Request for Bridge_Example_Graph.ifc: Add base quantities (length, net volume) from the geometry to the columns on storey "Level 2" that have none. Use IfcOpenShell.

First a look at what the model holds.

```python
import ifcopenshell
import ifcopenshell.util.element
import ifcopenshell.util.unit

model = ifcopenshell.open("Bridge_Example_Graph.ifc")
print(model.schema)
for unit_type in ("LENGTHUNIT", "AREAUNIT", "VOLUMEUNIT"):
    print(unit_type, ifcopenshell.util.unit.calculate_unit_scale(model, unit_type))
storey = next(s for s in model.by_type("IfcBuildingStorey") if s.Name == "Level 2")
columns = [e for e in ifcopenshell.util.element.get_decomposition(storey) if e.is_a("IfcColumn")]
for e in sorted(columns, key=lambda e: e.id()):
    print(e.id(), e.is_a(), e.Name, list(ifcopenshell.util.element.get_psets(e, qtos_only=True)), sep=" | ")
```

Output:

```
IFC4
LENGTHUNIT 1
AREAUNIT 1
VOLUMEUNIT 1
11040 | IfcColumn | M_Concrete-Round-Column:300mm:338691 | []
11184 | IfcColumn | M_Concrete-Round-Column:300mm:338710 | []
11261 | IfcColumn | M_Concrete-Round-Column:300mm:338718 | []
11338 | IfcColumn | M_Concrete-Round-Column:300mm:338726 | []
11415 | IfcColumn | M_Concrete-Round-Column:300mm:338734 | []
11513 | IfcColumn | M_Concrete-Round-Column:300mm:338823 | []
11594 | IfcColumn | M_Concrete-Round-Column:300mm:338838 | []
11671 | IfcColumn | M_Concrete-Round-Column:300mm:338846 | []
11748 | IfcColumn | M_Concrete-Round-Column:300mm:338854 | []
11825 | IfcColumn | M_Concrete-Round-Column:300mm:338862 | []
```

```python
import ifcopenshell
import ifcopenshell.api.pset
import ifcopenshell.geom
import ifcopenshell.util.element
import ifcopenshell.util.shape
import ifcopenshell.util.unit

model = ifcopenshell.open("Bridge_Example_Graph.ifc")
unit_scale = ifcopenshell.util.unit.calculate_unit_scale(model)
volume_scale = ifcopenshell.util.unit.calculate_unit_scale(model, "VOLUMEUNIT")
settings = ifcopenshell.geom.settings()

storey = next(s for s in model.by_type("IfcBuildingStorey") if s.Name == "Level 2")
columns = [e for e in ifcopenshell.util.element.get_decomposition(storey) if e.is_a("IfcColumn")]

for e in sorted(columns, key=lambda e: e.id()):
    if ifcopenshell.util.element.get_psets(e, qtos_only=True, should_inherit=False):
        continue
    # Geometry comes back in metres, in the element's own axes.
    shape = ifcopenshell.geom.create_shape(settings, e)
    values = {
        "Length": ifcopenshell.util.shape.get_z(shape.geometry) / unit_scale,
        "NetVolume": ifcopenshell.util.shape.get_volume(shape.geometry) / volume_scale,
    }
    qto = ifcopenshell.api.pset.add_qto(model, product=e, name="Qto_ColumnBaseQuantities")
    ifcopenshell.api.pset.edit_qto(model, qto=qto, properties=values)
    print(e.id(), {k: round(v, 3) for k, v in values.items()})

model.write("Bridge_Example_Graph-out.ifc")
```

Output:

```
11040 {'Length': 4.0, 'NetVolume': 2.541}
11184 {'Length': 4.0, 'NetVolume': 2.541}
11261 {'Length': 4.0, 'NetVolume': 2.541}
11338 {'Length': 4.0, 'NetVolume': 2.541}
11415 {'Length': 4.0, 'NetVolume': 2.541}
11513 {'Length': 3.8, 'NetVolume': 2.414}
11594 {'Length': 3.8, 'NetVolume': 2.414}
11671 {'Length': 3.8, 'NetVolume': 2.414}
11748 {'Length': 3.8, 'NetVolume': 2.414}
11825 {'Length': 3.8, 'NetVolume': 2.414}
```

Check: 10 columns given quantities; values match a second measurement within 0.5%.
